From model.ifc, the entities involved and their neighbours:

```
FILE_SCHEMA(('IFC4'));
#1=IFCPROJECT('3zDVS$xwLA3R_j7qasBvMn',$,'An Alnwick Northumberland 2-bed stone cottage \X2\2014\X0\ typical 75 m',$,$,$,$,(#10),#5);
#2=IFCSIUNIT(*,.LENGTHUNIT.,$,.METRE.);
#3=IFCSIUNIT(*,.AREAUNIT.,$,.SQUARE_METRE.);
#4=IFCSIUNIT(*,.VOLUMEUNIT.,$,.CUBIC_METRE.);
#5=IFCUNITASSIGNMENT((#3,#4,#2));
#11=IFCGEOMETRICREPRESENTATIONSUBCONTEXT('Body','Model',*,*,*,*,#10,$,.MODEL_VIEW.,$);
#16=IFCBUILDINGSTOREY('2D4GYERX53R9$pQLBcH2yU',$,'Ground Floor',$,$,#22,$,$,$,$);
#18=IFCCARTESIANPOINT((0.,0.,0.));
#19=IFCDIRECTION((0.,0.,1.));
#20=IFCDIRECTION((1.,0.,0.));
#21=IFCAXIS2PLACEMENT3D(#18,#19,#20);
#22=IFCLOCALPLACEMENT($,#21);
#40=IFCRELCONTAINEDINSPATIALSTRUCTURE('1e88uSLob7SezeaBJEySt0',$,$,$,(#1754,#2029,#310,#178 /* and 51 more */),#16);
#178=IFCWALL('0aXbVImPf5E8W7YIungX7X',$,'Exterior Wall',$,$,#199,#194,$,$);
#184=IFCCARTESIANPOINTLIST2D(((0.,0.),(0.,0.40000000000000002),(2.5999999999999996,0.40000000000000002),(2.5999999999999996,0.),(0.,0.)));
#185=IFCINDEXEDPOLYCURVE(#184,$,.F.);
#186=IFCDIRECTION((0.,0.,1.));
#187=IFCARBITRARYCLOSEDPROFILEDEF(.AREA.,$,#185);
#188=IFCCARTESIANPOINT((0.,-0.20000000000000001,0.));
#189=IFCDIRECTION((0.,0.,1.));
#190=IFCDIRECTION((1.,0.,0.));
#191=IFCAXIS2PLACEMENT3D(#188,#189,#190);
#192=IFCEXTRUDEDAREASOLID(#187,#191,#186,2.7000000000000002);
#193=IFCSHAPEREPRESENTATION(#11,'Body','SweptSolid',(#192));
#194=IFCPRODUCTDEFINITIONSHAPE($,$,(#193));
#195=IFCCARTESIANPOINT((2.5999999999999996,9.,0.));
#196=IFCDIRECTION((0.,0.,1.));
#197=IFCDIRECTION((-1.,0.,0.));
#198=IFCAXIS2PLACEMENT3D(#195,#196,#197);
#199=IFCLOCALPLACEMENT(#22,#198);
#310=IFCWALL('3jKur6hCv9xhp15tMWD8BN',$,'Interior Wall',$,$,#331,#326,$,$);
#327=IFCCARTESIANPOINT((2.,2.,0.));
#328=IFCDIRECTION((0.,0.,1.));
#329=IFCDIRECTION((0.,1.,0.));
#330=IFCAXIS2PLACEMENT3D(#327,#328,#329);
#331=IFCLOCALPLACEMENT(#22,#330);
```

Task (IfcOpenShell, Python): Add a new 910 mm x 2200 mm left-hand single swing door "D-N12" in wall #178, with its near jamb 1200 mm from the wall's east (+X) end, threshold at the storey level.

```python
import numpy as np
import ifcopenshell
import ifcopenshell.api.feature
import ifcopenshell.api.geometry
import ifcopenshell.api.root
import ifcopenshell.api.spatial
import ifcopenshell.geom
import ifcopenshell.util.element
import ifcopenshell.util.placement
import ifcopenshell.util.representation
import ifcopenshell.util.shape
import ifcopenshell.util.unit

model = ifcopenshell.open("model.ifc")
unit_scale = ifcopenshell.util.unit.calculate_unit_scale(model)
settings = ifcopenshell.geom.settings()


def volume(element):
    """Net volume in cubic metres, openings subtracted."""
    shape = ifcopenshell.geom.create_shape(settings, element)
    return ifcopenshell.util.shape.get_volume(shape.geometry)


wall = model.by_guid("0aXbVImPf5E8W7YIungX7X")
storey = ifcopenshell.util.element.get_container(wall, ifc_class="IfcBuildingStorey")
context = ifcopenshell.util.representation.get_context(model, "Model", "Body", "MODEL_VIEW")
before = volume(wall)

width, height, from_end, sill = 0.91, 2.2, 1.2, 0.0  # metres

# The wall runs along its own X axis, and the end named is its -X end.
wall_shape = ifcopenshell.geom.create_shape(settings, wall)
x, y, z = ifcopenshell.util.shape.get_vertices(wall_shape.geometry).T
start = x.min() + from_end
face, thickness = float(y.min()), float(y.max() - y.min())
wall_matrix = ifcopenshell.util.placement.get_local_placement(wall.ObjectPlacement)
level = ifcopenshell.util.placement.get_local_placement(storey.ObjectPlacement)[2, 3]


def in_wall(x, y):
    """Placement at x, y metres in the wall's axes, at sill height."""
    matrix = wall_matrix.copy()
    matrix[:, 3] = wall_matrix @ np.array([x / unit_scale, y / unit_scale, 0.0, 1.0])
    matrix[2, 3] = level + sill / unit_scale
    return matrix


# Opening: a box that overshoots both wall faces by 50 mm.
opening = ifcopenshell.api.root.create_entity(model, ifc_class="IfcOpeningElement", predefined_type="OPENING")
box = ifcopenshell.api.geometry.add_wall_representation(
    model, context=context, length=width, height=height, thickness=thickness + 0.1
)
ifcopenshell.api.geometry.assign_representation(model, product=opening, representation=box)
ifcopenshell.api.geometry.edit_object_placement(model, product=opening, matrix=in_wall(start, face - 0.05), is_si=False)
ifcopenshell.api.feature.add_feature(model, feature=opening, element=wall)

door = ifcopenshell.api.root.create_entity(model, ifc_class="IfcDoor", name="D-N12", predefined_type="DOOR")
door.OverallWidth, door.OverallHeight = width / unit_scale, height / unit_scale
door.OperationType = "SINGLE_SWING_LEFT"
body = ifcopenshell.api.geometry.add_door_representation(
    model,
    context=context,
    overall_width=door.OverallWidth,
    overall_height=door.OverallHeight,
    operation_type="SINGLE_SWING_LEFT",
    lining_properties={"LiningDepth": thickness / unit_scale, "ThresholdDepth": thickness / unit_scale},
)
ifcopenshell.api.geometry.assign_representation(model, product=door, representation=body)
ifcopenshell.api.spatial.assign_container(model, products=[door], relating_structure=storey)
ifcopenshell.api.feature.add_filling(model, opening=opening, element=door)

# The lining spans the wall, so the door starts at the wall face.
ifcopenshell.api.geometry.edit_object_placement(model, product=door, matrix=in_wall(start, face), is_si=False)

after = volume(wall)

print(f"wall volume {before:.3f} -> {after:.3f} m3")

model.write("model_v2.ifc")
```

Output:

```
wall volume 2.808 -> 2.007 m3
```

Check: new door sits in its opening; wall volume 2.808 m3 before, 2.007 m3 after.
